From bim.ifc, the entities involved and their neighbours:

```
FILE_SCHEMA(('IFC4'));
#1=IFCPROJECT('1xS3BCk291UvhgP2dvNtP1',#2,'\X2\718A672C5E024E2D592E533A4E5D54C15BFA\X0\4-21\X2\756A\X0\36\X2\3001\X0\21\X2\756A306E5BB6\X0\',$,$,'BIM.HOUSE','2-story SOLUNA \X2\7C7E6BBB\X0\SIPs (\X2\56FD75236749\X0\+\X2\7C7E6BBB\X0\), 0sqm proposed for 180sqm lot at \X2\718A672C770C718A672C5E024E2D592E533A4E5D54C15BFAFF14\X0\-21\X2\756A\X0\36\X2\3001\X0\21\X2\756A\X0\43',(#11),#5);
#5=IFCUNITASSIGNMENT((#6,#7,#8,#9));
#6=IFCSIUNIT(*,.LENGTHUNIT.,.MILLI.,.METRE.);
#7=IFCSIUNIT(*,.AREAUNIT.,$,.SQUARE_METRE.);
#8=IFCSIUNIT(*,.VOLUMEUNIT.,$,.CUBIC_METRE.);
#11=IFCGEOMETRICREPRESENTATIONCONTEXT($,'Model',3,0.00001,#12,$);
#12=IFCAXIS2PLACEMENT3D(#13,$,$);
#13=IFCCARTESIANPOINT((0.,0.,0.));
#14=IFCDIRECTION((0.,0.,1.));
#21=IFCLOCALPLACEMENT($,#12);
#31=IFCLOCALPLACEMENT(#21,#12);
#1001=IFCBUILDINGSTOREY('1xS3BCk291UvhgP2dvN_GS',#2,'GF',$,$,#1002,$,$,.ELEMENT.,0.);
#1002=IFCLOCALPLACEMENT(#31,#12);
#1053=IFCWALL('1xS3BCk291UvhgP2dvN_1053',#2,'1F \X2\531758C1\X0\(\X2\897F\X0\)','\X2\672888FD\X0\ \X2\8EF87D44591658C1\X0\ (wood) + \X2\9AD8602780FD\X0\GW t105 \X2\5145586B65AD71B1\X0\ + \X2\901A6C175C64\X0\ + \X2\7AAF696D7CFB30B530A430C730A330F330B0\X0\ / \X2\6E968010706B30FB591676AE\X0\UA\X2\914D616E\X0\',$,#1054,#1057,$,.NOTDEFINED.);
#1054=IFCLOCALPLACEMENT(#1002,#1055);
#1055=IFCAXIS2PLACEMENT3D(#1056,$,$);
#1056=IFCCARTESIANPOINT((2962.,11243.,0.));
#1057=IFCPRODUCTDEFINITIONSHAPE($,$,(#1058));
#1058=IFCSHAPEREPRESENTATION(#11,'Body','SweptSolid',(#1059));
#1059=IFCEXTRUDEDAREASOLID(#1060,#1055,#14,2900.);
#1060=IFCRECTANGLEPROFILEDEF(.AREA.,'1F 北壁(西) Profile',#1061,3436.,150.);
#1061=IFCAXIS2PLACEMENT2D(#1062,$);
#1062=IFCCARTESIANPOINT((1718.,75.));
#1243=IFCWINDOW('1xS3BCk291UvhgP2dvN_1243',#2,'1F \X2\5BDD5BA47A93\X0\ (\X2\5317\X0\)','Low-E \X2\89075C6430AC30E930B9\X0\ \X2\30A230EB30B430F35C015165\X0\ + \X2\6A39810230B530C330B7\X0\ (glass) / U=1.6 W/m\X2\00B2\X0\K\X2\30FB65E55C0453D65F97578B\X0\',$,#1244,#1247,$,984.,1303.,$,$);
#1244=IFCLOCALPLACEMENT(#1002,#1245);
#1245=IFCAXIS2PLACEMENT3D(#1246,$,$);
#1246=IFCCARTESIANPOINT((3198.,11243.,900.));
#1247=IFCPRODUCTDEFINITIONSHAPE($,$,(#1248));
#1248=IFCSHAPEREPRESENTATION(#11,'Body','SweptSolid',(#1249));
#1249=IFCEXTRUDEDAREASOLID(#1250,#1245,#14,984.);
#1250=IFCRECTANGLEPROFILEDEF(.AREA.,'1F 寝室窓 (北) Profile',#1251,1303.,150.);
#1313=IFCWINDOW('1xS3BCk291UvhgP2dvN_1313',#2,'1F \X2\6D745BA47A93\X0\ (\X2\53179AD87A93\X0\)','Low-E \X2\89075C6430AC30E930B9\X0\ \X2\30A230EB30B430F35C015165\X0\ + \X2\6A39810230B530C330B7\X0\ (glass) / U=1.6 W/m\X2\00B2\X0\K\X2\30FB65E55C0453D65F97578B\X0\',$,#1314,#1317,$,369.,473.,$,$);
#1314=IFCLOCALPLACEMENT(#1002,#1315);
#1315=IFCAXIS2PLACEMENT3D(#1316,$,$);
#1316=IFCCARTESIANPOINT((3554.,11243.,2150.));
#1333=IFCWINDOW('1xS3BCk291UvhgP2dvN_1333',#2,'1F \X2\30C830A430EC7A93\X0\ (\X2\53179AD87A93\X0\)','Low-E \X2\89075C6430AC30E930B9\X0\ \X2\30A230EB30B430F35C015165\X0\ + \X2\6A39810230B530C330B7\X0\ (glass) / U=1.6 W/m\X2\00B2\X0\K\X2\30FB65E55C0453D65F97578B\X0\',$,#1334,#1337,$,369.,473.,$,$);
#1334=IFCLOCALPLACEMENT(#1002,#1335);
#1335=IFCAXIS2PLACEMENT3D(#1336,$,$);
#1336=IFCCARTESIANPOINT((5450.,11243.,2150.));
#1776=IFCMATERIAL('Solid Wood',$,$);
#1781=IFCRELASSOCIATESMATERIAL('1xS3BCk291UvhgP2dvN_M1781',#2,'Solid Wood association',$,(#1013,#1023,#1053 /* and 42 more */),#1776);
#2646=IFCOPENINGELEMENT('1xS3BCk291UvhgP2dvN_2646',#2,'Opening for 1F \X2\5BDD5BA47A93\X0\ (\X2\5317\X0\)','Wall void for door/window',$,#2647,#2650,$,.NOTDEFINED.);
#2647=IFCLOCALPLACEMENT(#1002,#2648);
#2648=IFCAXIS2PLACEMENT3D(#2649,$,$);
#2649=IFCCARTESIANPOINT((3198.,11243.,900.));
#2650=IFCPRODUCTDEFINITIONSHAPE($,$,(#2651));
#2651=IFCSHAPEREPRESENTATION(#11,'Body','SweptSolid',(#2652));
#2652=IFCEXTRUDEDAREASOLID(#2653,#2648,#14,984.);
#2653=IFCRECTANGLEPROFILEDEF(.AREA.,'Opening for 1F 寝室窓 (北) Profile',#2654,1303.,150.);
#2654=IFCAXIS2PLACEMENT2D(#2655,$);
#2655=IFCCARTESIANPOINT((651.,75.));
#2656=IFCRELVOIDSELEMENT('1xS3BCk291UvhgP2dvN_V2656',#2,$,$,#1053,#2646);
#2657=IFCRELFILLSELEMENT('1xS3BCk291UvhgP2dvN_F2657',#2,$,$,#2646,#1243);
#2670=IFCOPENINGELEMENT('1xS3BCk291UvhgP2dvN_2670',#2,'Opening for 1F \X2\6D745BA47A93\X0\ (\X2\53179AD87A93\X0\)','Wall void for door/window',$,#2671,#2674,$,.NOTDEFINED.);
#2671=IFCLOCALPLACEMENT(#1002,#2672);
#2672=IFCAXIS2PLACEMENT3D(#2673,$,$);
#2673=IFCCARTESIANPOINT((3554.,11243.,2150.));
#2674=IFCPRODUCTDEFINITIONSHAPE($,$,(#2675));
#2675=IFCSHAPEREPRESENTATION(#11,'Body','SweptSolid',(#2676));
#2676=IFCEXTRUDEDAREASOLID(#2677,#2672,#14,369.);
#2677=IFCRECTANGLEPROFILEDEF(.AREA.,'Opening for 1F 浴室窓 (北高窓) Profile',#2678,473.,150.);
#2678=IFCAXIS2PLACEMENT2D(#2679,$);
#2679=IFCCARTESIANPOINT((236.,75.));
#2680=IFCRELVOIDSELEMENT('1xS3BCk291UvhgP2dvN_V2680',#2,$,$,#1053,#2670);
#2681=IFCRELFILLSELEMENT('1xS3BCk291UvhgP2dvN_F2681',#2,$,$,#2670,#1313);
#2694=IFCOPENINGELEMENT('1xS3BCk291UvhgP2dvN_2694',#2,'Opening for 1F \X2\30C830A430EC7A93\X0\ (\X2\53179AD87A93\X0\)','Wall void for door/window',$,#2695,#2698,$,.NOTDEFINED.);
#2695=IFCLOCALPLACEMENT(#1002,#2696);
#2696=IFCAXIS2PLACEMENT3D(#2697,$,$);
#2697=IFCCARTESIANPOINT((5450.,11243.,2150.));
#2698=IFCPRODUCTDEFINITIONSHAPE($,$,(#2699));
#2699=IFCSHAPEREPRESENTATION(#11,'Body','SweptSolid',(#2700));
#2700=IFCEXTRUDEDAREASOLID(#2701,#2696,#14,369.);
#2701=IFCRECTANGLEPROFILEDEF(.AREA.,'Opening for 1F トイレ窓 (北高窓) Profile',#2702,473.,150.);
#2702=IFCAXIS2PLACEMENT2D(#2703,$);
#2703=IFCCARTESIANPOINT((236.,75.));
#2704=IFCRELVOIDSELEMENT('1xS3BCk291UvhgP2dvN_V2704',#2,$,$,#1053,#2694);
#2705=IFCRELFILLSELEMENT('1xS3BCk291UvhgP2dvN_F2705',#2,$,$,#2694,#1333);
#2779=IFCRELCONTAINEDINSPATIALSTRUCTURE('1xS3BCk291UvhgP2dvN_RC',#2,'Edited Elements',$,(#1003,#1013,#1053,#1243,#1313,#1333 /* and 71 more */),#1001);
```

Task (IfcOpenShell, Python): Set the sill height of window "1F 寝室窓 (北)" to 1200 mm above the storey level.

```python
import numpy as np
import ifcopenshell
import ifcopenshell.api.geometry
import ifcopenshell.geom
import ifcopenshell.util.element
import ifcopenshell.util.placement
import ifcopenshell.util.shape
import ifcopenshell.util.unit

model = ifcopenshell.open("bim.ifc")
unit_scale = ifcopenshell.util.unit.calculate_unit_scale(model)

window = model.by_guid("1xS3BCk291UvhgP2dvN_1243")
opening = window.FillsVoids[0].RelatingOpeningElement
storey = ifcopenshell.util.element.get_container(window, ifc_class="IfcBuildingStorey")
level = ifcopenshell.util.placement.get_local_placement(storey.ObjectPlacement)[2, 3]

# The opening's origin need not be at the sill, so measure its lowest point.
shape = ifcopenshell.geom.create_shape(ifcopenshell.geom.settings(), opening)
bottom = ifcopenshell.util.shape.get_shape_bottom_elevation(shape, shape.geometry) / unit_scale
dz = level + 1.2 / unit_scale - bottom

shift = np.array([0.0, 0.0, dz])
# The window is not placed relative to its opening, so move both.
for product in (opening, window):
    matrix = ifcopenshell.util.placement.get_local_placement(product.ObjectPlacement)
    matrix[:3, 3] += shift
    ifcopenshell.api.geometry.edit_object_placement(model, product=product, matrix=matrix, is_si=False)

print(f"moved by {dz * unit_scale:+.3f} m")

model.write("bim_edited.ifc")
```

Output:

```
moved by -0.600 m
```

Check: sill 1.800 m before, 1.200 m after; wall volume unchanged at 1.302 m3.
